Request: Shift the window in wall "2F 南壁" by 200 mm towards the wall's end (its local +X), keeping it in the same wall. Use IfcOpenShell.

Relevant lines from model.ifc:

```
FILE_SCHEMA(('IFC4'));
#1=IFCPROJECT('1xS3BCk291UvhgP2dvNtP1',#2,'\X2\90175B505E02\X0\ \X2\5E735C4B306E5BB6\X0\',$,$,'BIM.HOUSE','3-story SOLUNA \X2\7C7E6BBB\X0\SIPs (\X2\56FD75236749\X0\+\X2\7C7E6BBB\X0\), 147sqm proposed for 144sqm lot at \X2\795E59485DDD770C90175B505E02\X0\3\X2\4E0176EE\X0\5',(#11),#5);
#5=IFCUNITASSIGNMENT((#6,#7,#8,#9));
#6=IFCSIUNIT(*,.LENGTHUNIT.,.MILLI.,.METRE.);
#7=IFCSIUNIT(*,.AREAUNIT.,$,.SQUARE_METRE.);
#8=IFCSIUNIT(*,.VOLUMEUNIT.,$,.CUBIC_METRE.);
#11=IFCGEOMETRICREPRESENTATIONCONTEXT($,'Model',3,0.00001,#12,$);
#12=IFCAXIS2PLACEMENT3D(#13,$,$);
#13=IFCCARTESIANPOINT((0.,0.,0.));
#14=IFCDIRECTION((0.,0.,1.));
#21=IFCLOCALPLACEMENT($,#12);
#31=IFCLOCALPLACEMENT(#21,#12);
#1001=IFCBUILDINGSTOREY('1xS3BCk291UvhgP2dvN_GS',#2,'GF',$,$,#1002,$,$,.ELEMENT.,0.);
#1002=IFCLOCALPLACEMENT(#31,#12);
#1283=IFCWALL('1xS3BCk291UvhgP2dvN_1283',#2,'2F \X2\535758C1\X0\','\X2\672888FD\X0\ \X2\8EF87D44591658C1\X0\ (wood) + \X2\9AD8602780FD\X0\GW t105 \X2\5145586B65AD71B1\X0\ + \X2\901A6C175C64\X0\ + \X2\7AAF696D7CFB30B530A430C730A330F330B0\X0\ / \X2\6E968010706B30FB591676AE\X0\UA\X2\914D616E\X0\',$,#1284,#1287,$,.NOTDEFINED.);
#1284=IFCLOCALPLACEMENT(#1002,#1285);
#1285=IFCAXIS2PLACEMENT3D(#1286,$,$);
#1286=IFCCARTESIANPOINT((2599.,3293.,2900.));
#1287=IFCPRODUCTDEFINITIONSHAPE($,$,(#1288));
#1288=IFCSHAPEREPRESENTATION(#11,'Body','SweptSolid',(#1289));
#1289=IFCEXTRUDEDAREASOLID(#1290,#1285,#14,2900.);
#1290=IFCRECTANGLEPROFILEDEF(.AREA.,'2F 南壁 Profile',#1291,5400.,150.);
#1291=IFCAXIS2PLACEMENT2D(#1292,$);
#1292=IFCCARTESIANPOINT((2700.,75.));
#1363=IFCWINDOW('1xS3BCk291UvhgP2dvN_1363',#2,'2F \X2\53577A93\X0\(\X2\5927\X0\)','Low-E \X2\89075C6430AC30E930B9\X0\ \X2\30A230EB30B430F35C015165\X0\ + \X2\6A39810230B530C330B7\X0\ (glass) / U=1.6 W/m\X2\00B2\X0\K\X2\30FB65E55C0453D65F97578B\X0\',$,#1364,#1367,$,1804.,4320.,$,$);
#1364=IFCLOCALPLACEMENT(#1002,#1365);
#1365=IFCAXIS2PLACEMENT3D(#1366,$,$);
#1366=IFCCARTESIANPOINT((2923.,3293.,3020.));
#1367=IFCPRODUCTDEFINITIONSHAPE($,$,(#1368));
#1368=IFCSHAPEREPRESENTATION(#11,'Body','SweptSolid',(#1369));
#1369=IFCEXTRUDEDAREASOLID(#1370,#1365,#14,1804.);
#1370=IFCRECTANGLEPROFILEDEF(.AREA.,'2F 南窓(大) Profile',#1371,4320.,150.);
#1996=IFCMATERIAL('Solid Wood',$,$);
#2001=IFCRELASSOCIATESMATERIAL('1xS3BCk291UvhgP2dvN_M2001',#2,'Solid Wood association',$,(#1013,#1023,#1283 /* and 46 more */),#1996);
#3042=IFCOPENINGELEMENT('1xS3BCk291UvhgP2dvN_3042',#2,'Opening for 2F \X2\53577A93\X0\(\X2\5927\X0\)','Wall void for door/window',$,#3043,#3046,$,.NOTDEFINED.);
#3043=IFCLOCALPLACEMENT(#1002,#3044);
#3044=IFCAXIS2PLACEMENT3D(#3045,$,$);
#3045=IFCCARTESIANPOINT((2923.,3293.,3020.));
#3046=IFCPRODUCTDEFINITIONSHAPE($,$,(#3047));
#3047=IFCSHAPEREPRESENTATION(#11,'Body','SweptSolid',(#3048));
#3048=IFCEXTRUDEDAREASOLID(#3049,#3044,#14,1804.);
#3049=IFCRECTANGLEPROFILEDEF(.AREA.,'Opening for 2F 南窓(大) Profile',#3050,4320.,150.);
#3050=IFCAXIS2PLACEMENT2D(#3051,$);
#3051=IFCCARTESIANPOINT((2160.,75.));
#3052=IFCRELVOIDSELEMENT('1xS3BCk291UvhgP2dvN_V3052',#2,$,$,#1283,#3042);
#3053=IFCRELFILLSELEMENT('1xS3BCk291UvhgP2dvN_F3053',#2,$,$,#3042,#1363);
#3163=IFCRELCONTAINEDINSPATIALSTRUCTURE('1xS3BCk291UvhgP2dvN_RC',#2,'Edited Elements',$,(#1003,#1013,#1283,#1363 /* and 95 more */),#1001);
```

```python
import ifcopenshell
import ifcopenshell.api.geometry
import ifcopenshell.util.placement

model = ifcopenshell.open("model.ifc")

window = model.by_guid("1xS3BCk291UvhgP2dvN_1363")
opening = window.FillsVoids[0].RelatingOpeningElement
wall = opening.VoidsElements[0].RelatingBuildingElement

wall_matrix = ifcopenshell.util.placement.get_local_placement(wall.ObjectPlacement)
shift = wall_matrix[:3, 0] * 200.0
before = ifcopenshell.util.placement.get_local_placement(window.ObjectPlacement)[:3, 3].copy()

# The window is not placed relative to its opening, so move both.
for product in (opening, window):
    matrix = ifcopenshell.util.placement.get_local_placement(product.ObjectPlacement)
    matrix[:3, 3] += shift
    ifcopenshell.api.geometry.edit_object_placement(model, product=product, matrix=matrix, is_si=False)

after = ifcopenshell.util.placement.get_local_placement(window.ObjectPlacement)[:3, 3]
print("window moved by", (after - before).round(3) + 0.0)

model.write("model_edited.ifc")
```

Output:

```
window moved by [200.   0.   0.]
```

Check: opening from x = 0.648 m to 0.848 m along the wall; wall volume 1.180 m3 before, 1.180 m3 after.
